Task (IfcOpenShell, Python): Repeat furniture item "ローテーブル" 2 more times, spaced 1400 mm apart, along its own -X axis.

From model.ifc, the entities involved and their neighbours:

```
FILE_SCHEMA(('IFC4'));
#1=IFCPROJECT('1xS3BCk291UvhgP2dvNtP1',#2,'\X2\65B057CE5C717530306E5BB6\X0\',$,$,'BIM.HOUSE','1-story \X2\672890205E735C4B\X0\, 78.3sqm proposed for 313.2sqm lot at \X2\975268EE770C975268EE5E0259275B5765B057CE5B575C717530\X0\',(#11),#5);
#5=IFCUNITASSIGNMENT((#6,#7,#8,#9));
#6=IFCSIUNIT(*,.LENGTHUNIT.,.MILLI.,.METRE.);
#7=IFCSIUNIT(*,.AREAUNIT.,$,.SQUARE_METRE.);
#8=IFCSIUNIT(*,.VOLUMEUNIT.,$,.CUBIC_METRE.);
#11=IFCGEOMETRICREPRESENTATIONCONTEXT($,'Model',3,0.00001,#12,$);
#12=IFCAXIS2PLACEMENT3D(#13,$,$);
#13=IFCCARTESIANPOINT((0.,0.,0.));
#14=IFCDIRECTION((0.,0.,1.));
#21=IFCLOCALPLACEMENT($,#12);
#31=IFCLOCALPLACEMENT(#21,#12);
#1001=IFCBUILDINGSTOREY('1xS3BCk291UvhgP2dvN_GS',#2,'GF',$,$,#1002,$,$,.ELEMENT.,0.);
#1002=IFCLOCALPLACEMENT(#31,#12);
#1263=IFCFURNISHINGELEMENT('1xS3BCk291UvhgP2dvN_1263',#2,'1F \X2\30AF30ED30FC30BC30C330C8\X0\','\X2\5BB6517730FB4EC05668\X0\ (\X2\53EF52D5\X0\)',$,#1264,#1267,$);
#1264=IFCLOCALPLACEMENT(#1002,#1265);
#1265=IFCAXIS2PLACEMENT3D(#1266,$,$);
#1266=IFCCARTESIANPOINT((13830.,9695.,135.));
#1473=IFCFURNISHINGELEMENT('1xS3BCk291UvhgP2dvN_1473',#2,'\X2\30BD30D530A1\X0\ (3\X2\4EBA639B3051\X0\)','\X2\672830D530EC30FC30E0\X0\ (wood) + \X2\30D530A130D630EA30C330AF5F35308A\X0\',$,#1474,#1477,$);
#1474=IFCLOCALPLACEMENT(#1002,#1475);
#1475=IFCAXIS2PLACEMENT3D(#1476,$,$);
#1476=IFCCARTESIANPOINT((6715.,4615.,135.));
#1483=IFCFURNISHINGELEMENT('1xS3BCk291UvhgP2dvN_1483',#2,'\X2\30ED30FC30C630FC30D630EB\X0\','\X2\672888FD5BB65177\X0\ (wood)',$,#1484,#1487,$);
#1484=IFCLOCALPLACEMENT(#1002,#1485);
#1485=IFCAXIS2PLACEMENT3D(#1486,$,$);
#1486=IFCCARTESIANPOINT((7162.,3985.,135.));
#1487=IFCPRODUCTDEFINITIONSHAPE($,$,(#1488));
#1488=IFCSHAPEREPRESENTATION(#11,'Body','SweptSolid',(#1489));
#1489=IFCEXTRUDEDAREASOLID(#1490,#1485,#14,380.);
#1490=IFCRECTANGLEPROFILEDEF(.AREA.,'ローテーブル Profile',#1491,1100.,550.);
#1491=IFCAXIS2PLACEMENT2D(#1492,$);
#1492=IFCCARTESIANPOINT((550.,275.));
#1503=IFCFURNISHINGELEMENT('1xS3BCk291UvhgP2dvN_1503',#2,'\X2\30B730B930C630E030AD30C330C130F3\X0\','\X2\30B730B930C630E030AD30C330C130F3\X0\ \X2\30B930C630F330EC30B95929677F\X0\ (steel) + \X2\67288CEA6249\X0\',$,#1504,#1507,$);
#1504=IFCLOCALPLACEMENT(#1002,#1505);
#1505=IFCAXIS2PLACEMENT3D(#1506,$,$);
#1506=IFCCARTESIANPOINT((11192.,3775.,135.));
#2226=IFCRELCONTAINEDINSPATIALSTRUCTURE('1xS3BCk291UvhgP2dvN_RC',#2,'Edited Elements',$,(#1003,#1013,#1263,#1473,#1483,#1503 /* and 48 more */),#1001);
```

```python
import ifcopenshell
import ifcopenshell.api.geometry
import ifcopenshell.api.root
import ifcopenshell.util.element
import ifcopenshell.util.placement
import ifcopenshell.util.unit

model = ifcopenshell.open("model.ifc")
unit_scale = ifcopenshell.util.unit.calculate_unit_scale(model)


def reuse_history(source, copy):
    """copy_class also copies each property set's owner history, people and application; keep the originals."""
    for rel in copy.IsDefinedBy:
        if rel.is_a("IfcRelDefinesByProperties") and (history := rel.RelatingPropertyDefinition.OwnerHistory):
            rel.RelatingPropertyDefinition.OwnerHistory = source.OwnerHistory
            ifcopenshell.util.element.remove_deep2(model, history)


source = model.by_guid("1xS3BCk291UvhgP2dvN_1483")
base = ifcopenshell.util.placement.get_local_placement(source.ObjectPlacement)
step = -base[:3, 0] * 1.4 / unit_scale

for i in range(1, 3):
    copy = ifcopenshell.api.root.copy_class(model, product=source)
    copy.Representation = ifcopenshell.util.element.copy_deep(
        model, source.Representation, exclude=["IfcGeometricRepresentationContext", "IfcRepresentationMap"]
    )
    reuse_history(source, copy)
    matrix = base.copy()
    matrix[:3, 3] += i * step
    print("added at", matrix[:3, 3].round(3) + 0.0)
    ifcopenshell.api.geometry.edit_object_placement(model, product=copy, matrix=matrix, is_si=False)

model.write("model_updated.ifc")
```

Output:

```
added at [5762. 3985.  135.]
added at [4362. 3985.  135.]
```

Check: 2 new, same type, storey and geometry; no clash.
